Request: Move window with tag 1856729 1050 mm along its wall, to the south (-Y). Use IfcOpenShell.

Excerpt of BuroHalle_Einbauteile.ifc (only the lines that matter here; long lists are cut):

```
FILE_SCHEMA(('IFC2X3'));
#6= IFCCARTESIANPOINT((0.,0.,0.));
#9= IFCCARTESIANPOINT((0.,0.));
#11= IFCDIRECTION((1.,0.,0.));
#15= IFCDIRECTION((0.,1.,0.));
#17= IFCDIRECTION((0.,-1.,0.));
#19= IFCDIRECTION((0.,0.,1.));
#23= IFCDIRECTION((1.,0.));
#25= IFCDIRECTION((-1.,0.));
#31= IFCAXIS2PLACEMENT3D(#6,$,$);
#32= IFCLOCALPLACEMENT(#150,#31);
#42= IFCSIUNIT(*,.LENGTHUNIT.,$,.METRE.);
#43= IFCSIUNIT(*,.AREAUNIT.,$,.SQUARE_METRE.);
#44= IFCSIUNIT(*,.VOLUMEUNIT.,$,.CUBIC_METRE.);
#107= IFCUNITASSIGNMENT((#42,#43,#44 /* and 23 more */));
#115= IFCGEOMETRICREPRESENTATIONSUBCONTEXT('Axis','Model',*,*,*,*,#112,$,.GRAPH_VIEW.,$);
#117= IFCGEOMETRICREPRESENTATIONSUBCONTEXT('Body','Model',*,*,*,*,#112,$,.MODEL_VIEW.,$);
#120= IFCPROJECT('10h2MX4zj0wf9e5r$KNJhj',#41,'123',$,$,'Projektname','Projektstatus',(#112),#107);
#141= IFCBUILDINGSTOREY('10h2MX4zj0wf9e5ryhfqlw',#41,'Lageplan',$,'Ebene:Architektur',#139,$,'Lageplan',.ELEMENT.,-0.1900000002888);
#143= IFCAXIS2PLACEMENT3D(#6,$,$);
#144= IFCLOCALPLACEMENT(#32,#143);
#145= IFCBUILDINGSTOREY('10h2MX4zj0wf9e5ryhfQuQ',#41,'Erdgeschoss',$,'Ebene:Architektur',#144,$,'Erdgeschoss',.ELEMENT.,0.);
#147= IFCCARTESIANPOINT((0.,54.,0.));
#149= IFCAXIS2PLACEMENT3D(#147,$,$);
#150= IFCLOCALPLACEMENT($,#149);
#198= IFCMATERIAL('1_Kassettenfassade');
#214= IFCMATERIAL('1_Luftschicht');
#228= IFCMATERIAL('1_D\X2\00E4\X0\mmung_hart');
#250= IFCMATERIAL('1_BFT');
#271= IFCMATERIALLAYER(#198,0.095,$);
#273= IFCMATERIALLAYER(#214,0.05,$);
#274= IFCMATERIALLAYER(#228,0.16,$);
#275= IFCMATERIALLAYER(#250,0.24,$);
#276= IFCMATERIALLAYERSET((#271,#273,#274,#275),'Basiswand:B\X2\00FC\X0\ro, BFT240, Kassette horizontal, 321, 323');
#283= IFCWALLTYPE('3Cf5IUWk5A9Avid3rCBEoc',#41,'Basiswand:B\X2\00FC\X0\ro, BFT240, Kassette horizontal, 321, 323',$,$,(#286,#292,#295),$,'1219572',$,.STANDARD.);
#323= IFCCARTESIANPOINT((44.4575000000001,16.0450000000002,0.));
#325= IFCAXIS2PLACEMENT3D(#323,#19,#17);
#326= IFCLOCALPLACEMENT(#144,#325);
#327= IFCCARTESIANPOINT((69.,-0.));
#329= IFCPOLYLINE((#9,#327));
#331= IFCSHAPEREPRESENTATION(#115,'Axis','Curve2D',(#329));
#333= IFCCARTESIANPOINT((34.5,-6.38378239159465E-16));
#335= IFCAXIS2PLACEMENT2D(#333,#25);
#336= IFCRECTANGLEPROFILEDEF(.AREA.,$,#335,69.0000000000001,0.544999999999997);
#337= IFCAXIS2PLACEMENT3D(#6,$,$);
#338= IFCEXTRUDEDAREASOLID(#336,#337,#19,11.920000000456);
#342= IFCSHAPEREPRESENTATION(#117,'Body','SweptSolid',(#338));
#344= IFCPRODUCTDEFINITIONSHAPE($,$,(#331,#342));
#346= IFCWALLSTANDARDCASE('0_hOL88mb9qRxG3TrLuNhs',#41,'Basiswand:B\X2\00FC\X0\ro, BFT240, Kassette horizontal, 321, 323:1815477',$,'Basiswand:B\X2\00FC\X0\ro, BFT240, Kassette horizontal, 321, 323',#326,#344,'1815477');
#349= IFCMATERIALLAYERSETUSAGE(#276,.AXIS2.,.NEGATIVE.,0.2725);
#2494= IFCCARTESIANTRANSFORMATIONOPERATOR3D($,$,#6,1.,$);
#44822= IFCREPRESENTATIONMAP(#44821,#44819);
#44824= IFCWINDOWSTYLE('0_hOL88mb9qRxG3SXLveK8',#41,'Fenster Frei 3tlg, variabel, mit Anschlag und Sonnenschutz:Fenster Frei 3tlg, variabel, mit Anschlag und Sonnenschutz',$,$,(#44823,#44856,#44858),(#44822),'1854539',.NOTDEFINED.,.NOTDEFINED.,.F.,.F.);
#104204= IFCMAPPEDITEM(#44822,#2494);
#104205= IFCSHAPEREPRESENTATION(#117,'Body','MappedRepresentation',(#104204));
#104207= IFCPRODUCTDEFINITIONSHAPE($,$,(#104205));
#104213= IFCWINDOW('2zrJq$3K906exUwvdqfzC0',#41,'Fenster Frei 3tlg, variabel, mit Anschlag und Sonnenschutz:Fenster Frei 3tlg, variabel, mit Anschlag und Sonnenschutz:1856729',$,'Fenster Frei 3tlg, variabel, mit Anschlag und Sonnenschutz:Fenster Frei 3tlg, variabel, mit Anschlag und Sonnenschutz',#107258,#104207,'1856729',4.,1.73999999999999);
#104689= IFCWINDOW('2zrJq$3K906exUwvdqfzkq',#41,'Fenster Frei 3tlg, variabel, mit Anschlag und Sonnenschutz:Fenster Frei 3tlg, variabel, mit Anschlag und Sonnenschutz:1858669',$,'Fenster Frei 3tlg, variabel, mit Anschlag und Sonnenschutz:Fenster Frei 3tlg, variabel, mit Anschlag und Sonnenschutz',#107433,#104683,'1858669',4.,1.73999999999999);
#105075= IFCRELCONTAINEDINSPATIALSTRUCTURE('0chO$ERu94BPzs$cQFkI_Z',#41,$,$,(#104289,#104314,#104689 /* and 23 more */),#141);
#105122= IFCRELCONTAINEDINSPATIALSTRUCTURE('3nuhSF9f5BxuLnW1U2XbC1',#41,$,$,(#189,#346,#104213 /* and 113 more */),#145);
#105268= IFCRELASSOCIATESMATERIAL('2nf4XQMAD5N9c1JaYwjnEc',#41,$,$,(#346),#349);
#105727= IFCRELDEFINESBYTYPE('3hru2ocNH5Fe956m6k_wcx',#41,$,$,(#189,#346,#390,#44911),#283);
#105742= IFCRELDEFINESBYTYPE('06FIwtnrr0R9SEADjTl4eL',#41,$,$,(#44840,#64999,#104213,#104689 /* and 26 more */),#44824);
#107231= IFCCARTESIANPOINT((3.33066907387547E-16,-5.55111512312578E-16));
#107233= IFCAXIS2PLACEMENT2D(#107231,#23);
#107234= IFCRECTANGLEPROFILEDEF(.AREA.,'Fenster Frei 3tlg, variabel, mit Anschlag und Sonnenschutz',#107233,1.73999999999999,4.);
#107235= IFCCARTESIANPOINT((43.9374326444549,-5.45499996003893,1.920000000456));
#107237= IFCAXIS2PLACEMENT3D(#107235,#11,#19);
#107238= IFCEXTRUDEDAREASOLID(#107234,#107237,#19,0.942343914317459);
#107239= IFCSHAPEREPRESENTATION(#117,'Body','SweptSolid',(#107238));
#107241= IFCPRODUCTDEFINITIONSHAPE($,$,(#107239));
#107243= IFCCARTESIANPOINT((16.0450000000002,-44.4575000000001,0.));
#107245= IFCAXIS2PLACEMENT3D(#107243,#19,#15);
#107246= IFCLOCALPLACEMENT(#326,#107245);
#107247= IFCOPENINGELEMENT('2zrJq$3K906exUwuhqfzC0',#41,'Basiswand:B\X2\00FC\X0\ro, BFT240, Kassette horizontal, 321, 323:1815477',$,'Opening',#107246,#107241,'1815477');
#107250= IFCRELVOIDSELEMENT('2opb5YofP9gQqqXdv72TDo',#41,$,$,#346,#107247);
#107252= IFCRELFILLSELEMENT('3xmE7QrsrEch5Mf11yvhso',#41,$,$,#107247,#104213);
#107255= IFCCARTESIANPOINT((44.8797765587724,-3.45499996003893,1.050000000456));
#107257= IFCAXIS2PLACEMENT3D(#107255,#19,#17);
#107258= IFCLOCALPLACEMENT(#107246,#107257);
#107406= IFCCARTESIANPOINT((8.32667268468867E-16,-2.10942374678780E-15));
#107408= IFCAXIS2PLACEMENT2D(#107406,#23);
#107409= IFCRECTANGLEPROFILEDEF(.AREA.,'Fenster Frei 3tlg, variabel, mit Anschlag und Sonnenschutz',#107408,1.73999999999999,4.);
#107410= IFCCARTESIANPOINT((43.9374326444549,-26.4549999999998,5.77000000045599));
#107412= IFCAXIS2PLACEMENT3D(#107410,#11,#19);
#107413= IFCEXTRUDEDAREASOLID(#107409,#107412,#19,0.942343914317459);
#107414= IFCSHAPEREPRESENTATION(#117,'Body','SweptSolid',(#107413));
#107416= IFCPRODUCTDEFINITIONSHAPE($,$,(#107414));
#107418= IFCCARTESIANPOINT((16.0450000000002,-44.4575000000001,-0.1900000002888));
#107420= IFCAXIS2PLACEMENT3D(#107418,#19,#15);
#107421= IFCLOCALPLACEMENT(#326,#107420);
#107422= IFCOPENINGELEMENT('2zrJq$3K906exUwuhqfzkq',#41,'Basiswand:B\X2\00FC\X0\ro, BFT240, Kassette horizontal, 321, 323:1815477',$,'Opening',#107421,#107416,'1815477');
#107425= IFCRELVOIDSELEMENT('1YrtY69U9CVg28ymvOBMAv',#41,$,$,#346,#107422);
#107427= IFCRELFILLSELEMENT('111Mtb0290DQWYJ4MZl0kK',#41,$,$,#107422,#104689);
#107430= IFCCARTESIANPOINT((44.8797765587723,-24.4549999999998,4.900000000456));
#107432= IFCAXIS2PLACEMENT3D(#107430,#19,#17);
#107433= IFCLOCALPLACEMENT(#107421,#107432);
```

```python
import ifcopenshell
import ifcopenshell.api.geometry
import ifcopenshell.util.placement
import ifcopenshell.util.unit

model = ifcopenshell.open("BuroHalle_Einbauteile.ifc")
unit_scale = ifcopenshell.util.unit.calculate_unit_scale(model)

window = model.by_id(104213)
opening = window.FillsVoids[0].RelatingOpeningElement
wall = opening.VoidsElements[0].RelatingBuildingElement

wall_matrix = ifcopenshell.util.placement.get_local_placement(wall.ObjectPlacement)
shift = wall_matrix[:3, 0] * 1.05 / unit_scale
before = ifcopenshell.util.placement.get_local_placement(window.ObjectPlacement)[:3, 3].copy()

# The window is placed relative to its opening, so it follows when the opening moves.
matrix = ifcopenshell.util.placement.get_local_placement(opening.ObjectPlacement)
matrix[:3, 3] += shift
ifcopenshell.api.geometry.edit_object_placement(
    model, product=opening, matrix=matrix, is_si=False, should_transform_children=True
)

after = ifcopenshell.util.placement.get_local_placement(window.ObjectPlacement)[:3, 3]
print("window moved by", (after - before).round(3) + 0.0)

model.write("BuroHalle_Einbauteile_rev.ifc")
```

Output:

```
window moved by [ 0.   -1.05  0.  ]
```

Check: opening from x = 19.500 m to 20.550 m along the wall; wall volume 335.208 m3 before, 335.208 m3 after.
